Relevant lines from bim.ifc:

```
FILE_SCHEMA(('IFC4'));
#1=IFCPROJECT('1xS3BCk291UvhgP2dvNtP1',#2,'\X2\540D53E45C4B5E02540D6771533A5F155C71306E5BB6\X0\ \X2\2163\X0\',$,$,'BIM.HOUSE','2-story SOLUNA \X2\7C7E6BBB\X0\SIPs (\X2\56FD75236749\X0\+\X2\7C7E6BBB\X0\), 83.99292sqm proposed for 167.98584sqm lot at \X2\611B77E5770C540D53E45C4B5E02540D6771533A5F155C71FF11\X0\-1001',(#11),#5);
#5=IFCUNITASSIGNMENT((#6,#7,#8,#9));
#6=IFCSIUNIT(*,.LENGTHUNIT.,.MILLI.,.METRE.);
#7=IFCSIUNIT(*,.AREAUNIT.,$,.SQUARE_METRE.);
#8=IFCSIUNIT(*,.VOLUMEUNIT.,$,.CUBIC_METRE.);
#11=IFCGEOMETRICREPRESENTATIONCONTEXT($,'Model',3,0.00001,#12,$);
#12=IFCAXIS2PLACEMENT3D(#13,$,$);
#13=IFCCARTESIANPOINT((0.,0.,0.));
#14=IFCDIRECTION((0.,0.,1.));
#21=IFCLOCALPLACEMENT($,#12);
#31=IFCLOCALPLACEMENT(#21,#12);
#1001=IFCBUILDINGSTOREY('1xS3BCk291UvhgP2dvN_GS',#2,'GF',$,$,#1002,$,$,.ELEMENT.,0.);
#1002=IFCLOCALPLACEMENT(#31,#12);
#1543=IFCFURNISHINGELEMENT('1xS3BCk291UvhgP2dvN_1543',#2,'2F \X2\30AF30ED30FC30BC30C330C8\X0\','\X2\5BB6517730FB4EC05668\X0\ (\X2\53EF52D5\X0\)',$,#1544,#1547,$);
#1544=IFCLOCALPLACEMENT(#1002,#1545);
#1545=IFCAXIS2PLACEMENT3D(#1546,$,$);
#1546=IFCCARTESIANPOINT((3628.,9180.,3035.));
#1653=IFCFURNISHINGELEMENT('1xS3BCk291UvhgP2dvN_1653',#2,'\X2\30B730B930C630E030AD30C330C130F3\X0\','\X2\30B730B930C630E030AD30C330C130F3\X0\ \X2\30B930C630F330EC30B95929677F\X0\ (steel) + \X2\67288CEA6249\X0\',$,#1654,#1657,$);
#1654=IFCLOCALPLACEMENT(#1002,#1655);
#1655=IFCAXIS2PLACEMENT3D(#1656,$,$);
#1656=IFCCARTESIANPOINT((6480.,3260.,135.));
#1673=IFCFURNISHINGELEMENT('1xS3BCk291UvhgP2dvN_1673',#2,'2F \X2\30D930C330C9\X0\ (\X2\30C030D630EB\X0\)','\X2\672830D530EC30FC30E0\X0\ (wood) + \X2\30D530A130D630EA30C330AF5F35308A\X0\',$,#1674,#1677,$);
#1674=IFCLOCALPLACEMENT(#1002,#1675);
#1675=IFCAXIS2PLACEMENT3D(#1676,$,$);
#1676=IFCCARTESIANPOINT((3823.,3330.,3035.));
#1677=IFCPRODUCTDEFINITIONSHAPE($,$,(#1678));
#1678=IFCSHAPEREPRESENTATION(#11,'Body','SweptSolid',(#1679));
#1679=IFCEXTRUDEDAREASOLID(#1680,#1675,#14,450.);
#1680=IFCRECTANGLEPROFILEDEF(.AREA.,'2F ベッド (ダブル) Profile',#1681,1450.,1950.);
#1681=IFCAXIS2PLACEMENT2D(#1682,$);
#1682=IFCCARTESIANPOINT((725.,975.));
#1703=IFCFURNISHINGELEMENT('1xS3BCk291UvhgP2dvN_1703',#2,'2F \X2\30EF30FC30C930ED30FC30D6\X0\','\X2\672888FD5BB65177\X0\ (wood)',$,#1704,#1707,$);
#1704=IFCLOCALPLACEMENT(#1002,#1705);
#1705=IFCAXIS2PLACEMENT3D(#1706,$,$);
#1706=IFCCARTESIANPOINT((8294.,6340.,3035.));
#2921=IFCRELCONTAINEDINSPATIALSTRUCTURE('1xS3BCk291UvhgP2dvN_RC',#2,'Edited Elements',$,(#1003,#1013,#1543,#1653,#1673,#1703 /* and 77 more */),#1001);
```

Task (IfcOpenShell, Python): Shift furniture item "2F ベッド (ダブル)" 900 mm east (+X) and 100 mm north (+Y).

```python
import ifcopenshell
import ifcopenshell.api.geometry
import ifcopenshell.util.placement
import ifcopenshell.util.unit

model = ifcopenshell.open("bim.ifc")
unit_scale = ifcopenshell.util.unit.calculate_unit_scale(model)

item = model.by_id(1673)
matrix = ifcopenshell.util.placement.get_local_placement(item.ObjectPlacement)
matrix[0, 3] += 0.9 / unit_scale
matrix[1, 3] += 0.1 / unit_scale
ifcopenshell.api.geometry.edit_object_placement(model, product=item, matrix=matrix, is_si=False)

print(ifcopenshell.util.placement.get_local_placement(item.ObjectPlacement).round(3) + 0.0)

model.write("bim_rev.ifc")
```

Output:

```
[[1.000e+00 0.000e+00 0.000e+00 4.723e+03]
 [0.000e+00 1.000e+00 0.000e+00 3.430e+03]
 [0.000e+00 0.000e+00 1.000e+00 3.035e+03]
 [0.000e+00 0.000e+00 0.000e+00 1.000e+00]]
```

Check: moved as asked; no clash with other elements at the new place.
